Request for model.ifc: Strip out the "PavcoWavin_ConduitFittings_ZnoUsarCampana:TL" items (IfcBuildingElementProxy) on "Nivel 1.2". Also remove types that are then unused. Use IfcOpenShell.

First a look at what the model holds.

```python
import ifcopenshell
import ifcopenshell.util.element

model = ifcopenshell.open("model.ifc")
print(model.schema)
storey = next(s for s in model.by_type("IfcBuildingStorey") if s.Name == "Nivel 1.2")
proxies = [e for e in ifcopenshell.util.element.get_decomposition(storey) if e.is_a("IfcBuildingElementProxy")]
seen = {}
for e in proxies:
    element_type = ifcopenshell.util.element.get_type(e)
    name = element_type.Name if element_type not in (None, e) else None
    seen[name] = seen.get(name, 0) + 1
for name, count in sorted(seen.items(), key=str):
    print(count, "x", name)
```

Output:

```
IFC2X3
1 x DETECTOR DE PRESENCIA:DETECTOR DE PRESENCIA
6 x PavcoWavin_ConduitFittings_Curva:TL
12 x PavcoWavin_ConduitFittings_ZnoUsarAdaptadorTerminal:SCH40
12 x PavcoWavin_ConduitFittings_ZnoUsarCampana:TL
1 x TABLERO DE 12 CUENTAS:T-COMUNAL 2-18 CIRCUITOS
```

```python
import ifcopenshell
import ifcopenshell.api.root
import ifcopenshell.util.element

model = ifcopenshell.open("model.ifc")

storey = next(s for s in model.by_type("IfcBuildingStorey") if s.Name == "Nivel 1.2")
proxies = [e for e in ifcopenshell.util.element.get_decomposition(storey) if e.is_a("IfcBuildingElementProxy")]
targets = [e for e in proxies if (t := ifcopenshell.util.element.get_type(e)) not in (None, e) and t.Name == "PavcoWavin_ConduitFittings_ZnoUsarCampana:TL"]
types = {ifcopenshell.util.element.get_type(e) for e in targets} - {None, *targets}

for e in targets:
    ifcopenshell.api.root.remove_product(model, product=e)
print(len(targets), "removed")

unused = [t for t in types if not ifcopenshell.util.element.get_types(t)]
for t in unused:
    ifcopenshell.api.root.remove_product(model, product=t)
print(len(unused), "unused types removed")

model.write("model_edited.ifc")
```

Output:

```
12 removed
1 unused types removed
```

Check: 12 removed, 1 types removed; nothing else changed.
